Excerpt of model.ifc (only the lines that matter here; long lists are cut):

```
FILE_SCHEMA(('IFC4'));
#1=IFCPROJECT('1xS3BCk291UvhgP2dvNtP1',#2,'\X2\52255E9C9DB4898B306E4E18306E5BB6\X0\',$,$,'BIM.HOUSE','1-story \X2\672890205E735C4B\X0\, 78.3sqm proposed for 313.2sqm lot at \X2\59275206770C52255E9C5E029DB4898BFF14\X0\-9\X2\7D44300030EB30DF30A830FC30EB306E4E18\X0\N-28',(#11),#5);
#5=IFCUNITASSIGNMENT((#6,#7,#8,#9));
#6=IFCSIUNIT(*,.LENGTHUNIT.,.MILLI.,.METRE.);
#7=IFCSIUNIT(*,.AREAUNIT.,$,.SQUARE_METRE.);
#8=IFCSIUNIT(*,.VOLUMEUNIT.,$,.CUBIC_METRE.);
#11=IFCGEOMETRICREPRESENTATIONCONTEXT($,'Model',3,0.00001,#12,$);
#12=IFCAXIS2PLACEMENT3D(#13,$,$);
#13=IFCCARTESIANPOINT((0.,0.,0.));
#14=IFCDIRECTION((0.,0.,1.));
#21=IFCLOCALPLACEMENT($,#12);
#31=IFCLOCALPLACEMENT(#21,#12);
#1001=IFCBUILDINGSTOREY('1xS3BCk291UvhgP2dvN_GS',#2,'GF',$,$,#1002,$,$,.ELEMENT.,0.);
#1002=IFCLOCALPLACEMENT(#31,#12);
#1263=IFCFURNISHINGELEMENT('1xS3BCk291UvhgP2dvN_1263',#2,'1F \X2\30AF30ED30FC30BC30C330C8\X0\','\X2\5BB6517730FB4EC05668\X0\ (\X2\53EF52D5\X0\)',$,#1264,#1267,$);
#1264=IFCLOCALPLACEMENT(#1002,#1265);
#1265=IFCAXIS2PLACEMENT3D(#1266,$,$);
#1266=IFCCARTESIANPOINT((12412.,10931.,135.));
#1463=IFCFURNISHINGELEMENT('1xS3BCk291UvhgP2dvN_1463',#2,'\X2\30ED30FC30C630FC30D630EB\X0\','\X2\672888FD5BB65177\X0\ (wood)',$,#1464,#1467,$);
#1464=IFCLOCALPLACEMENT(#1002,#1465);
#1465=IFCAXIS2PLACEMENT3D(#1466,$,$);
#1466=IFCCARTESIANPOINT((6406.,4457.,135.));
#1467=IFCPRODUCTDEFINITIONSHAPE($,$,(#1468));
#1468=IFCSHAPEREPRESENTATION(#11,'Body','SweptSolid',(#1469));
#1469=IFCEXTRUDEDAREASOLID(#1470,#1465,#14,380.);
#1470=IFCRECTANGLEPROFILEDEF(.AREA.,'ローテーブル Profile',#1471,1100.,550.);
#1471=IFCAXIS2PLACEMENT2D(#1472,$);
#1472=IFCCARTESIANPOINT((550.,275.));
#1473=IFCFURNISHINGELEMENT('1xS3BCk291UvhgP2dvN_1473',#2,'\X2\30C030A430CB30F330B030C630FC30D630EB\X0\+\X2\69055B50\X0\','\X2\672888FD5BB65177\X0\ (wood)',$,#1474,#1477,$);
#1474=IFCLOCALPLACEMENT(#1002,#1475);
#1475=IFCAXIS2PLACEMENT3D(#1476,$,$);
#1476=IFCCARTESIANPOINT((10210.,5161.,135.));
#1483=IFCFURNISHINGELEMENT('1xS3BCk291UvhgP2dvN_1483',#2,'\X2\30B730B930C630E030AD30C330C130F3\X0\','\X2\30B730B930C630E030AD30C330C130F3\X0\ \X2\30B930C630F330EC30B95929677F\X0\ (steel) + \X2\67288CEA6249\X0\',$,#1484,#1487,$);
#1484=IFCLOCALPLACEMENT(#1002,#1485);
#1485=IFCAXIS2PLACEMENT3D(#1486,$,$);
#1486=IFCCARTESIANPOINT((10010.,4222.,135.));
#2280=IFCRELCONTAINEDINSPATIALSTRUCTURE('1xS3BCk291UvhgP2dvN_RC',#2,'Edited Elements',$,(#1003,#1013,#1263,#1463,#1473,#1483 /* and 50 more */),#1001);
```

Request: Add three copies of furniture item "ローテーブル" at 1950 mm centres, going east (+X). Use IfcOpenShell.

```python
import numpy as np
import ifcopenshell
import ifcopenshell.api.geometry
import ifcopenshell.api.root
import ifcopenshell.util.element
import ifcopenshell.util.placement

model = ifcopenshell.open("model.ifc")


def reuse_history(source, copy):
    """copy_class also copies each property set's owner history, people and application; keep the originals."""
    for rel in copy.IsDefinedBy:
        if rel.is_a("IfcRelDefinesByProperties") and (history := rel.RelatingPropertyDefinition.OwnerHistory):
            rel.RelatingPropertyDefinition.OwnerHistory = source.OwnerHistory
            ifcopenshell.util.element.remove_deep2(model, history)


source = model.by_guid("1xS3BCk291UvhgP2dvN_1463")
base = ifcopenshell.util.placement.get_local_placement(source.ObjectPlacement)
step = np.array([1.0, 0.0, 0.0]) * 1950.0

for i in range(1, 4):
    copy = ifcopenshell.api.root.copy_class(model, product=source)
    copy.Representation = ifcopenshell.util.element.copy_deep(
        model, source.Representation, exclude=["IfcGeometricRepresentationContext", "IfcRepresentationMap"]
    )
    reuse_history(source, copy)
    matrix = base.copy()
    matrix[:3, 3] += i * step
    print("added at", matrix[:3, 3].round(3) + 0.0)
    ifcopenshell.api.geometry.edit_object_placement(model, product=copy, matrix=matrix, is_si=False)

model.write("model_edited.ifc")
```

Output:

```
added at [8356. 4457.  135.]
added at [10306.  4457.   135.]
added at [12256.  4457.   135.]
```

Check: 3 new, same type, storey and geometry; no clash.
